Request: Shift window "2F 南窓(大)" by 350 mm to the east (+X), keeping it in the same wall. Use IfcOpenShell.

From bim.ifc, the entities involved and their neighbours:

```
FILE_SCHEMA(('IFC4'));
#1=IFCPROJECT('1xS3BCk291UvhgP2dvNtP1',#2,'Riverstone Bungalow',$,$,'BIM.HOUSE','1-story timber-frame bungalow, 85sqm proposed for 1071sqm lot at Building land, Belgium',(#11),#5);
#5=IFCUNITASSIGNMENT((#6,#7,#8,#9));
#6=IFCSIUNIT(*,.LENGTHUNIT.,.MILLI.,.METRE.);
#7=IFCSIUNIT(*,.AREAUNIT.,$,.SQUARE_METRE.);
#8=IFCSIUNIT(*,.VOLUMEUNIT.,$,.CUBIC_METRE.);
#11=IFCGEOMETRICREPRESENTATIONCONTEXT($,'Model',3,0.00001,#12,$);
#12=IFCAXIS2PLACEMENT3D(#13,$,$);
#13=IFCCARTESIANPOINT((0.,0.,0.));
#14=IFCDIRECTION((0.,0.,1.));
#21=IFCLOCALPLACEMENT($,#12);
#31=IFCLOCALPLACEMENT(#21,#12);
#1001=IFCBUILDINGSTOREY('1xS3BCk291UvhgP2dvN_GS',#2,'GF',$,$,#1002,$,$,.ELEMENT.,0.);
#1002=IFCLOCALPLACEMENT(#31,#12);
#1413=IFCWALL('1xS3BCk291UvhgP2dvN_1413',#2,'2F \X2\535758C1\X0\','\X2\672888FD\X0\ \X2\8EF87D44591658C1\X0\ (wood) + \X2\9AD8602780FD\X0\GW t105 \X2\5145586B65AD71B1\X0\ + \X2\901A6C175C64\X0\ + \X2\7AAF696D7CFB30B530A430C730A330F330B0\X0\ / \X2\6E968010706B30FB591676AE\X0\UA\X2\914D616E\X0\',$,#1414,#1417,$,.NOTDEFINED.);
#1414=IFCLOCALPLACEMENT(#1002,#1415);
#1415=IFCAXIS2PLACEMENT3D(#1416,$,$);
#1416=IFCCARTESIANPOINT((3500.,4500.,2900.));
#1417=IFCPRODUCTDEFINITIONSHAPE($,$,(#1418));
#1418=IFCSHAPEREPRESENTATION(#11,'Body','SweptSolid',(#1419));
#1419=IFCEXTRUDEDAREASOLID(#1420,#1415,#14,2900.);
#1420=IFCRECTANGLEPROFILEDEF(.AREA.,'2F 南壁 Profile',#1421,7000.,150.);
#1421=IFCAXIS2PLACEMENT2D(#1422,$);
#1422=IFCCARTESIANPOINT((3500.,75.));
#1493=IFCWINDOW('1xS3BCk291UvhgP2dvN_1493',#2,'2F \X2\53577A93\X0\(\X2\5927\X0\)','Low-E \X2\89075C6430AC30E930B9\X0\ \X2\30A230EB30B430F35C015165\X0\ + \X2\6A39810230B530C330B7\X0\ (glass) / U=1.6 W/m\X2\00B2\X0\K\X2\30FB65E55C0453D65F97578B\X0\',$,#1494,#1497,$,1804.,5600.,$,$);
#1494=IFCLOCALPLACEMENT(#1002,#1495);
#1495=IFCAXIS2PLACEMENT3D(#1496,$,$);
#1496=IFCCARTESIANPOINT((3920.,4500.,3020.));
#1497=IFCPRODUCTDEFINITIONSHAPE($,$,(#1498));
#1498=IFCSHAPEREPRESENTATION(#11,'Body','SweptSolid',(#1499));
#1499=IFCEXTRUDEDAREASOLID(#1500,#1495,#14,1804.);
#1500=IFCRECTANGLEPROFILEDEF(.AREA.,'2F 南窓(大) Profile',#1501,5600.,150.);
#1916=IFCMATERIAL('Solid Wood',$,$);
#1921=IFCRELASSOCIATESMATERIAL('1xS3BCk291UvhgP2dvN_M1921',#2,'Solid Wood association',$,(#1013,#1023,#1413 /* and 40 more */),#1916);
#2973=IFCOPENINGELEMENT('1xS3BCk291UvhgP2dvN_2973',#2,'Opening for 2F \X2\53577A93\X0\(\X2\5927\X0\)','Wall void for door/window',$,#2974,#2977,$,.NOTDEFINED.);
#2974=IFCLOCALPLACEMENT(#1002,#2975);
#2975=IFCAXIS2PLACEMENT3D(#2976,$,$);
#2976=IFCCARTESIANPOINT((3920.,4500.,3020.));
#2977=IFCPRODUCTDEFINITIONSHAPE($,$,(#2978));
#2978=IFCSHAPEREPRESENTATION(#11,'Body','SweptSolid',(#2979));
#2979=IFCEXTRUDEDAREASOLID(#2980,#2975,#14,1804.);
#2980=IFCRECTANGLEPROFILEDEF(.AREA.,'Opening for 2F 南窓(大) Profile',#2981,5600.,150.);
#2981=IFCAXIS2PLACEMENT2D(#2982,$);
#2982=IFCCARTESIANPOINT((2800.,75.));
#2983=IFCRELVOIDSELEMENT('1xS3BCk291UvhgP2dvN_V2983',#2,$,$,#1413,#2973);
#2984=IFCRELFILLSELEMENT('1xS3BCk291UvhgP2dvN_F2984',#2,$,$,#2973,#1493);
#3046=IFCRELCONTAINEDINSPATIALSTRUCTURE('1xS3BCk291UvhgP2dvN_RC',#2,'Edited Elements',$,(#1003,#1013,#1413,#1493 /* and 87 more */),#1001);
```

```python
import ifcopenshell
import ifcopenshell.api.geometry
import ifcopenshell.util.placement
import ifcopenshell.util.unit

model = ifcopenshell.open("bim.ifc")
unit_scale = ifcopenshell.util.unit.calculate_unit_scale(model)

window = model.by_guid("1xS3BCk291UvhgP2dvN_1493")
opening = window.FillsVoids[0].RelatingOpeningElement
wall = opening.VoidsElements[0].RelatingBuildingElement

wall_matrix = ifcopenshell.util.placement.get_local_placement(wall.ObjectPlacement)
shift = wall_matrix[:3, 0] * 0.35 / unit_scale
before = ifcopenshell.util.placement.get_local_placement(window.ObjectPlacement)[:3, 3].copy()

# The window is not placed relative to its opening, so move both.
for product in (opening, window):
    matrix = ifcopenshell.util.placement.get_local_placement(product.ObjectPlacement)
    matrix[:3, 3] += shift
    ifcopenshell.api.geometry.edit_object_placement(model, product=product, matrix=matrix, is_si=False)

after = ifcopenshell.util.placement.get_local_placement(window.ObjectPlacement)[:3, 3]
print("window moved by", (after - before).round(3) + 0.0)

model.write("bim_updated.ifc")
```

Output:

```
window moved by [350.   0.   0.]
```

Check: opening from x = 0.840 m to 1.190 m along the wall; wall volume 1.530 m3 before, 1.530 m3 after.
